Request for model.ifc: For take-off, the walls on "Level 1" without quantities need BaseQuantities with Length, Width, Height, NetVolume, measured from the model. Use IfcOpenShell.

First a look at what the model holds.

```python
import ifcopenshell
import ifcopenshell.util.element
import ifcopenshell.util.unit

model = ifcopenshell.open("model.ifc")
print(model.schema)
for unit_type in ("LENGTHUNIT", "AREAUNIT", "VOLUMEUNIT"):
    print(unit_type, ifcopenshell.util.unit.calculate_unit_scale(model, unit_type))
storey = next(s for s in model.by_type("IfcBuildingStorey") if s.Name == "Level 1")
walls = [e for e in ifcopenshell.util.element.get_decomposition(storey) if e.is_a("IfcWall")]
for e in sorted(walls, key=lambda e: e.id()):
    print(e.id(), e.is_a(), e.Name, list(ifcopenshell.util.element.get_psets(e, qtos_only=True)), sep=" | ")
```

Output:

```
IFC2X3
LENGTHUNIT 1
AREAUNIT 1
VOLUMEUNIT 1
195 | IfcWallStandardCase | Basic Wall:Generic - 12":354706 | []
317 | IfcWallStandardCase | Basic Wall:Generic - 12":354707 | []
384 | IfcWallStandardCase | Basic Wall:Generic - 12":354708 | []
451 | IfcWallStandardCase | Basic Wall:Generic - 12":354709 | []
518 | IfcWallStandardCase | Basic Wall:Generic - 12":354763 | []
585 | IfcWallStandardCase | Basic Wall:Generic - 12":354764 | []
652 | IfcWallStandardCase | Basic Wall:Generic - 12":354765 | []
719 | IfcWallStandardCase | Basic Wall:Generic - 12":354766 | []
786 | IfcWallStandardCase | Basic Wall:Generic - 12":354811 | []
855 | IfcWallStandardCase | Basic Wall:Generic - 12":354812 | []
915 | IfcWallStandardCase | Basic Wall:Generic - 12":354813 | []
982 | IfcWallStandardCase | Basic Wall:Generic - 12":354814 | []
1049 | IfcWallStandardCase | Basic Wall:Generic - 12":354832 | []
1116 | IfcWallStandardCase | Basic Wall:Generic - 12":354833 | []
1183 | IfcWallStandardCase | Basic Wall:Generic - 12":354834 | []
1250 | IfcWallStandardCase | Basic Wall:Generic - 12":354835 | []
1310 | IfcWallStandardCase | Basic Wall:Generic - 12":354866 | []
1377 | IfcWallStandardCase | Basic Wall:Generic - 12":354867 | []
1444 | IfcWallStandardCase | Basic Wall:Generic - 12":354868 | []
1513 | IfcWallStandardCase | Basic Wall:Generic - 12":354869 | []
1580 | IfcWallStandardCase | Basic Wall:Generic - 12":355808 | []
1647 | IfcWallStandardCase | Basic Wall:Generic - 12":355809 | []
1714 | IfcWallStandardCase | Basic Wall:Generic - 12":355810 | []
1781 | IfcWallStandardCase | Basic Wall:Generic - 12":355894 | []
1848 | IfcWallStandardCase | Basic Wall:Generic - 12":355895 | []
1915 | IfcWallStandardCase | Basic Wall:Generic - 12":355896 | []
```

```python
import ifcopenshell
import ifcopenshell.api.pset
import ifcopenshell.geom
import ifcopenshell.util.element
import ifcopenshell.util.shape
import ifcopenshell.util.unit

model = ifcopenshell.open("model.ifc")
unit_scale = ifcopenshell.util.unit.calculate_unit_scale(model)
volume_scale = ifcopenshell.util.unit.calculate_unit_scale(model, "VOLUMEUNIT")
settings = ifcopenshell.geom.settings()

storey = next(s for s in model.by_type("IfcBuildingStorey") if s.Name == "Level 1")
walls = [e for e in ifcopenshell.util.element.get_decomposition(storey) if e.is_a("IfcWall")]

for e in sorted(walls, key=lambda e: e.id()):
    if ifcopenshell.util.element.get_psets(e, qtos_only=True, should_inherit=False):
        continue
    # Geometry comes back in metres, in the element's own axes.
    shape = ifcopenshell.geom.create_shape(settings, e)
    values = {
        "Length": ifcopenshell.util.shape.get_x(shape.geometry) / unit_scale,
        "Width": ifcopenshell.util.shape.get_y(shape.geometry) / unit_scale,
        "Height": ifcopenshell.util.shape.get_z(shape.geometry) / unit_scale,
        "NetVolume": ifcopenshell.util.shape.get_volume(shape.geometry) / volume_scale,
    }
    qto = ifcopenshell.api.pset.add_qto(model, product=e, name="BaseQuantities")
    ifcopenshell.api.pset.edit_qto(model, qto=qto, properties=values)
    print(e.id(), {k: round(v, 3) for k, v in values.items()})

model.write("model_rev.ifc")
```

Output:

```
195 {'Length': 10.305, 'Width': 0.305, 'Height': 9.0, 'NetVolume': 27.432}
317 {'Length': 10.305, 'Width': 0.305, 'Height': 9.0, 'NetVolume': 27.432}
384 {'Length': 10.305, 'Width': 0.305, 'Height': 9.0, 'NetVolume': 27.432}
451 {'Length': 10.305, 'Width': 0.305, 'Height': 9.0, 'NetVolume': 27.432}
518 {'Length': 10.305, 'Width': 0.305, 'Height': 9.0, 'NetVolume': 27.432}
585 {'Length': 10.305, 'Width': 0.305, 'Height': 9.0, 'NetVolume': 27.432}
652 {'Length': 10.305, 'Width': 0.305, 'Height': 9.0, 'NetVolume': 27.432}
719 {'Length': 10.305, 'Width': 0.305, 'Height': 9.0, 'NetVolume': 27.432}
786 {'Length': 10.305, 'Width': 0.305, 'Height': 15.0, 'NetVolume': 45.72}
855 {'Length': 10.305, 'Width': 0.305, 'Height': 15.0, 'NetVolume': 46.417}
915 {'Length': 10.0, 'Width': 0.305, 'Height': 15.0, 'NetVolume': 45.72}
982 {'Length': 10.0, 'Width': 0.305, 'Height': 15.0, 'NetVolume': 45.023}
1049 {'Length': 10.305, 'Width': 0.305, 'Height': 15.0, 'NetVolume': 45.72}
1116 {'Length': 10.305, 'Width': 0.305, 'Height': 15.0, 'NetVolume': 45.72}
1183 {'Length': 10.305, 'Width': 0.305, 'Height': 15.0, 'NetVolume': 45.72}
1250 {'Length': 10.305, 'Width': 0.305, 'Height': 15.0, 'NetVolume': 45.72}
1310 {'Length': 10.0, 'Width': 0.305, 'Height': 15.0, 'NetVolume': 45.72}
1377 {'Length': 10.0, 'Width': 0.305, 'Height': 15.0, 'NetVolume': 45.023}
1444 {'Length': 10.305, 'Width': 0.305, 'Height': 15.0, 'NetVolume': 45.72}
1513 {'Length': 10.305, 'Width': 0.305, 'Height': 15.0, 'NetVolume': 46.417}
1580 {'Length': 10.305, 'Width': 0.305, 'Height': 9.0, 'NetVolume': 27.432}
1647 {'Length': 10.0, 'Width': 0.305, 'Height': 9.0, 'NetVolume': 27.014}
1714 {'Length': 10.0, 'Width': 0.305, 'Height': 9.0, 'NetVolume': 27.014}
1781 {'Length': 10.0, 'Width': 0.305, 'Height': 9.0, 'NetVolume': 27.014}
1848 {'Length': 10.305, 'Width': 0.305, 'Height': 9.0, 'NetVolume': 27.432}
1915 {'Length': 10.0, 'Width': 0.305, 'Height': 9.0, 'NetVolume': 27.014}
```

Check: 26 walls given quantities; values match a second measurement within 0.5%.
